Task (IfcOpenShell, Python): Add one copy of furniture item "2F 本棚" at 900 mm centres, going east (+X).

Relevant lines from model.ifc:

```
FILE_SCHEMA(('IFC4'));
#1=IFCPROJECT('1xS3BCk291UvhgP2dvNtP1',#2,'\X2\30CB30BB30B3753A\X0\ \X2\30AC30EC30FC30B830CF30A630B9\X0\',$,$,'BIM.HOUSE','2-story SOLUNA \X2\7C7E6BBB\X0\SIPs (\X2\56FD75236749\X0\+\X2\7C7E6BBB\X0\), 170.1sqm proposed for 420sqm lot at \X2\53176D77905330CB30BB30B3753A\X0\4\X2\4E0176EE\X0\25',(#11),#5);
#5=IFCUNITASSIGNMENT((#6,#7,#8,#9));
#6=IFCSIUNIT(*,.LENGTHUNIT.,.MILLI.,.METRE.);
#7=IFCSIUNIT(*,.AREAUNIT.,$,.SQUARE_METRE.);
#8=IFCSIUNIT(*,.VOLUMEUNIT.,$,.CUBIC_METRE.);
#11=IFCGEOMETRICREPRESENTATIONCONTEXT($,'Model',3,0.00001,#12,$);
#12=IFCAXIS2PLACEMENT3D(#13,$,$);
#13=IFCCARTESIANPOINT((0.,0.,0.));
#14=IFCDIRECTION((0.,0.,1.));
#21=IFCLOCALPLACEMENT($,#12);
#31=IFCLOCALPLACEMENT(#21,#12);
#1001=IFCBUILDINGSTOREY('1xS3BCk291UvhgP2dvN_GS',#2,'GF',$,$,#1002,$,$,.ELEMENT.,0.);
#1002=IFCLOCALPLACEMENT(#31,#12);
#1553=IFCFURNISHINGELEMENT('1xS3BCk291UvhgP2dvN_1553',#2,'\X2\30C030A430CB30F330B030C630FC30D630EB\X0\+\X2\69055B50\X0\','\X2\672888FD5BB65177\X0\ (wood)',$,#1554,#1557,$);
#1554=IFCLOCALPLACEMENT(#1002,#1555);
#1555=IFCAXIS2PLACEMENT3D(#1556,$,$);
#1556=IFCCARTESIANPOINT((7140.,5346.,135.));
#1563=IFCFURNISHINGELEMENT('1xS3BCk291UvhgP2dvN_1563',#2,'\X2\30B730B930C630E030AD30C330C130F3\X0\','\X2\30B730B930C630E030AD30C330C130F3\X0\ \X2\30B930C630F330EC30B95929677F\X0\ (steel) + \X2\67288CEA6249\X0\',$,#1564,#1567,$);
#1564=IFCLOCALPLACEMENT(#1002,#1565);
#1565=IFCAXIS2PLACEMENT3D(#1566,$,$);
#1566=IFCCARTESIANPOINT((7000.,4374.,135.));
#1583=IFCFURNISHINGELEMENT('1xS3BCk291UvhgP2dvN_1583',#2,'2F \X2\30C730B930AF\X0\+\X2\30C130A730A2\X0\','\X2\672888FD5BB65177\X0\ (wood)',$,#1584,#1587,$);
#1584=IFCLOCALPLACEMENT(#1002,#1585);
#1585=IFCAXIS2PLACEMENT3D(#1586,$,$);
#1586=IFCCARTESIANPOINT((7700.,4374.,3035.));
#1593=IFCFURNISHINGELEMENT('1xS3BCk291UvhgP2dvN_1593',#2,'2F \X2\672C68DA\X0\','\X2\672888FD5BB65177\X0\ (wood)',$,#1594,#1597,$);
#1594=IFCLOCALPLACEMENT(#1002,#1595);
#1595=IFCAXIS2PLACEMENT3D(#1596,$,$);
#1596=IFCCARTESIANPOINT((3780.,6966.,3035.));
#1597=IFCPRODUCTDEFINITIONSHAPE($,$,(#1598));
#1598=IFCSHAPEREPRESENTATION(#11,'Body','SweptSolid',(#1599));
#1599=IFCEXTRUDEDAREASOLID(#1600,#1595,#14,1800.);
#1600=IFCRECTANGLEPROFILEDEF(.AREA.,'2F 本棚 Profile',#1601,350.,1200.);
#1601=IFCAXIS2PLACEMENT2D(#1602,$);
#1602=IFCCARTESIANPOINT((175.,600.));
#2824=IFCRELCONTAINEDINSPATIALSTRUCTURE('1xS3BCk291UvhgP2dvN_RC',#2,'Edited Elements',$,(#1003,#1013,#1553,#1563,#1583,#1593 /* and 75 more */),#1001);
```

```python
import numpy as np
import ifcopenshell
import ifcopenshell.api.geometry
import ifcopenshell.api.root
import ifcopenshell.util.element
import ifcopenshell.util.placement
import ifcopenshell.util.unit

model = ifcopenshell.open("model.ifc")
unit_scale = ifcopenshell.util.unit.calculate_unit_scale(model)


def reuse_history(source, copy):
    """copy_class also copies each property set's owner history, people and application; keep the originals."""
    for rel in copy.IsDefinedBy:
        if rel.is_a("IfcRelDefinesByProperties") and (history := rel.RelatingPropertyDefinition.OwnerHistory):
            rel.RelatingPropertyDefinition.OwnerHistory = source.OwnerHistory
            ifcopenshell.util.element.remove_deep2(model, history)


source = model.by_id(1593)
base = ifcopenshell.util.placement.get_local_placement(source.ObjectPlacement)
step = np.array([1.0, 0.0, 0.0]) * 0.9 / unit_scale

for i in range(1, 2):
    copy = ifcopenshell.api.root.copy_class(model, product=source)
    copy.Representation = ifcopenshell.util.element.copy_deep(
        model, source.Representation, exclude=["IfcGeometricRepresentationContext", "IfcRepresentationMap"]
    )
    reuse_history(source, copy)
    matrix = base.copy()
    matrix[:3, 3] += i * step
    print("added at", matrix[:3, 3].round(3) + 0.0)
    ifcopenshell.api.geometry.edit_object_placement(model, product=copy, matrix=matrix, is_si=False)

model.write("model_updated.ifc")
```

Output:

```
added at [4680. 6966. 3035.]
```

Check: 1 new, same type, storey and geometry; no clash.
